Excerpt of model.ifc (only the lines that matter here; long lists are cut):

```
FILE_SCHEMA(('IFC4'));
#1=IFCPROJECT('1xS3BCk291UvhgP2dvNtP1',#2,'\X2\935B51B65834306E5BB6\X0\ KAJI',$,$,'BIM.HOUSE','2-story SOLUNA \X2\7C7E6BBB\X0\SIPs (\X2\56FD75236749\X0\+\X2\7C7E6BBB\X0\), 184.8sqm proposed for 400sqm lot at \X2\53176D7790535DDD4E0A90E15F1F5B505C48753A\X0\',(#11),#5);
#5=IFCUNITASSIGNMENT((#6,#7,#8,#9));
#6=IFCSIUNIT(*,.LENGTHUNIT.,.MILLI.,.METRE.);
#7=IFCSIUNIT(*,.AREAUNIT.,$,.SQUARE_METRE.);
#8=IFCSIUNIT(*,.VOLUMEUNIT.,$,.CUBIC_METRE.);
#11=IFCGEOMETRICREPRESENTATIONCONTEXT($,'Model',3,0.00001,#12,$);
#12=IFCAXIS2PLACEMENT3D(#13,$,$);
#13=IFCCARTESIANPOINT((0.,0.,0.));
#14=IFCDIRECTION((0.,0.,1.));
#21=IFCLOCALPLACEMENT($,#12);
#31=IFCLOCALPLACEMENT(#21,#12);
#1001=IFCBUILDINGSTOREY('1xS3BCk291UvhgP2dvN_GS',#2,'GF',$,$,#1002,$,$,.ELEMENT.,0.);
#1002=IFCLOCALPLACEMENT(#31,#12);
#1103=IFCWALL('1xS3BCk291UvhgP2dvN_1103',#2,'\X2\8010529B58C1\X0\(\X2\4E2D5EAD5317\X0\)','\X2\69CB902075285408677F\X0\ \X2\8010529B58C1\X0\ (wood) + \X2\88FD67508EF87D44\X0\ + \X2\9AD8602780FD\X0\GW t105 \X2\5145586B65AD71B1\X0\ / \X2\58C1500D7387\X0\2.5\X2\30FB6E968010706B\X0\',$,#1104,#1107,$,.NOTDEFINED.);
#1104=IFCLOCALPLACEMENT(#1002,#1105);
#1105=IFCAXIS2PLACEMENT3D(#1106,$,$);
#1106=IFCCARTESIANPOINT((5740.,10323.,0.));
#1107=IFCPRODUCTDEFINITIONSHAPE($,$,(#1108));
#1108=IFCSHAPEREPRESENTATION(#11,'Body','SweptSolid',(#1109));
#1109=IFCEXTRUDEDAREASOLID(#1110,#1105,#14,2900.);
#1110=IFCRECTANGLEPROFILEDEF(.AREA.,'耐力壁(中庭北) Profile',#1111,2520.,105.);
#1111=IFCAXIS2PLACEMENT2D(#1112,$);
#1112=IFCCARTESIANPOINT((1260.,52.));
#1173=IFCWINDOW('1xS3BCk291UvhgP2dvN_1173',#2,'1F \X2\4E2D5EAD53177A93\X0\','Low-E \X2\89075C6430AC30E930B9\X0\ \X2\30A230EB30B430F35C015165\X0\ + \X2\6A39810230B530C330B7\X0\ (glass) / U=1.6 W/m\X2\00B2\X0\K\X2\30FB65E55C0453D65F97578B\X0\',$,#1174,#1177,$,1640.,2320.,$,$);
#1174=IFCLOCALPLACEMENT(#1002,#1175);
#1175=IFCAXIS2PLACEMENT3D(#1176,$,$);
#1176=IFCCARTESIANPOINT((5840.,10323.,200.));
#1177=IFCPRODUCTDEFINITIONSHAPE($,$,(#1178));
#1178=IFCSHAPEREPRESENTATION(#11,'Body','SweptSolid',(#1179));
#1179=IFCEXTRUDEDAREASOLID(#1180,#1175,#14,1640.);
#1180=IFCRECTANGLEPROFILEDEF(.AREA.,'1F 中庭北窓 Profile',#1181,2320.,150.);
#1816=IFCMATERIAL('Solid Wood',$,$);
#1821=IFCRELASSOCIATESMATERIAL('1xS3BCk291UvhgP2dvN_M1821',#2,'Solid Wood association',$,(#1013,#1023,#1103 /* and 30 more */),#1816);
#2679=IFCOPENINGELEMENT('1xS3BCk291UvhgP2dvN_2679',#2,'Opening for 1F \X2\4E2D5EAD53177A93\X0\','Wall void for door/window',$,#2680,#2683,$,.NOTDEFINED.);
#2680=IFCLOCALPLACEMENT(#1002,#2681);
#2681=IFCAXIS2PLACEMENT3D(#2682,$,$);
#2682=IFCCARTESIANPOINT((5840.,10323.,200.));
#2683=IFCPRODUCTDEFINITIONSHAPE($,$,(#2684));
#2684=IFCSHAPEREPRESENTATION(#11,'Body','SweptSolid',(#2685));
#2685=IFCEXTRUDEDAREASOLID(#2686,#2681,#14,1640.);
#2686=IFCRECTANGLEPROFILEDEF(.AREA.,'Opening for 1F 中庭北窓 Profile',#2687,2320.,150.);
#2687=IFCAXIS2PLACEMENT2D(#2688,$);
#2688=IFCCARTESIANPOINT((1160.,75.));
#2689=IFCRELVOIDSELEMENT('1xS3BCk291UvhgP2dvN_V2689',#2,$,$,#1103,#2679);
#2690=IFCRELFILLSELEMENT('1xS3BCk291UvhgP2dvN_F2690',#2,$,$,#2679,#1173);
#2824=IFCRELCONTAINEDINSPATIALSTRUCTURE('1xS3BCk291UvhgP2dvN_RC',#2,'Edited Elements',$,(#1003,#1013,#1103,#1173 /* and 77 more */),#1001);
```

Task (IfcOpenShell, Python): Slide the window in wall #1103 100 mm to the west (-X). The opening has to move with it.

```python
import ifcopenshell
import ifcopenshell.api.geometry
import ifcopenshell.util.placement
import ifcopenshell.util.unit

model = ifcopenshell.open("model.ifc")
unit_scale = ifcopenshell.util.unit.calculate_unit_scale(model)

window = model.by_id(1173)
opening = window.FillsVoids[0].RelatingOpeningElement
wall = opening.VoidsElements[0].RelatingBuildingElement

wall_matrix = ifcopenshell.util.placement.get_local_placement(wall.ObjectPlacement)
shift = wall_matrix[:3, 0] * -0.1 / unit_scale
before = ifcopenshell.util.placement.get_local_placement(window.ObjectPlacement)[:3, 3].copy()

# The window is not placed relative to its opening, so move both.
for product in (opening, window):
    matrix = ifcopenshell.util.placement.get_local_placement(product.ObjectPlacement)
    matrix[:3, 3] += shift
    ifcopenshell.api.geometry.edit_object_placement(model, product=product, matrix=matrix, is_si=False)

after = ifcopenshell.util.placement.get_local_placement(window.ObjectPlacement)[:3, 3]
print("window moved by", (after - before).round(3) + 0.0)

model.write("model_v2.ifc")
```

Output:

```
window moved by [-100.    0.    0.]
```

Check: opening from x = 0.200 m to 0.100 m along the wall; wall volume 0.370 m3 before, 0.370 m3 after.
